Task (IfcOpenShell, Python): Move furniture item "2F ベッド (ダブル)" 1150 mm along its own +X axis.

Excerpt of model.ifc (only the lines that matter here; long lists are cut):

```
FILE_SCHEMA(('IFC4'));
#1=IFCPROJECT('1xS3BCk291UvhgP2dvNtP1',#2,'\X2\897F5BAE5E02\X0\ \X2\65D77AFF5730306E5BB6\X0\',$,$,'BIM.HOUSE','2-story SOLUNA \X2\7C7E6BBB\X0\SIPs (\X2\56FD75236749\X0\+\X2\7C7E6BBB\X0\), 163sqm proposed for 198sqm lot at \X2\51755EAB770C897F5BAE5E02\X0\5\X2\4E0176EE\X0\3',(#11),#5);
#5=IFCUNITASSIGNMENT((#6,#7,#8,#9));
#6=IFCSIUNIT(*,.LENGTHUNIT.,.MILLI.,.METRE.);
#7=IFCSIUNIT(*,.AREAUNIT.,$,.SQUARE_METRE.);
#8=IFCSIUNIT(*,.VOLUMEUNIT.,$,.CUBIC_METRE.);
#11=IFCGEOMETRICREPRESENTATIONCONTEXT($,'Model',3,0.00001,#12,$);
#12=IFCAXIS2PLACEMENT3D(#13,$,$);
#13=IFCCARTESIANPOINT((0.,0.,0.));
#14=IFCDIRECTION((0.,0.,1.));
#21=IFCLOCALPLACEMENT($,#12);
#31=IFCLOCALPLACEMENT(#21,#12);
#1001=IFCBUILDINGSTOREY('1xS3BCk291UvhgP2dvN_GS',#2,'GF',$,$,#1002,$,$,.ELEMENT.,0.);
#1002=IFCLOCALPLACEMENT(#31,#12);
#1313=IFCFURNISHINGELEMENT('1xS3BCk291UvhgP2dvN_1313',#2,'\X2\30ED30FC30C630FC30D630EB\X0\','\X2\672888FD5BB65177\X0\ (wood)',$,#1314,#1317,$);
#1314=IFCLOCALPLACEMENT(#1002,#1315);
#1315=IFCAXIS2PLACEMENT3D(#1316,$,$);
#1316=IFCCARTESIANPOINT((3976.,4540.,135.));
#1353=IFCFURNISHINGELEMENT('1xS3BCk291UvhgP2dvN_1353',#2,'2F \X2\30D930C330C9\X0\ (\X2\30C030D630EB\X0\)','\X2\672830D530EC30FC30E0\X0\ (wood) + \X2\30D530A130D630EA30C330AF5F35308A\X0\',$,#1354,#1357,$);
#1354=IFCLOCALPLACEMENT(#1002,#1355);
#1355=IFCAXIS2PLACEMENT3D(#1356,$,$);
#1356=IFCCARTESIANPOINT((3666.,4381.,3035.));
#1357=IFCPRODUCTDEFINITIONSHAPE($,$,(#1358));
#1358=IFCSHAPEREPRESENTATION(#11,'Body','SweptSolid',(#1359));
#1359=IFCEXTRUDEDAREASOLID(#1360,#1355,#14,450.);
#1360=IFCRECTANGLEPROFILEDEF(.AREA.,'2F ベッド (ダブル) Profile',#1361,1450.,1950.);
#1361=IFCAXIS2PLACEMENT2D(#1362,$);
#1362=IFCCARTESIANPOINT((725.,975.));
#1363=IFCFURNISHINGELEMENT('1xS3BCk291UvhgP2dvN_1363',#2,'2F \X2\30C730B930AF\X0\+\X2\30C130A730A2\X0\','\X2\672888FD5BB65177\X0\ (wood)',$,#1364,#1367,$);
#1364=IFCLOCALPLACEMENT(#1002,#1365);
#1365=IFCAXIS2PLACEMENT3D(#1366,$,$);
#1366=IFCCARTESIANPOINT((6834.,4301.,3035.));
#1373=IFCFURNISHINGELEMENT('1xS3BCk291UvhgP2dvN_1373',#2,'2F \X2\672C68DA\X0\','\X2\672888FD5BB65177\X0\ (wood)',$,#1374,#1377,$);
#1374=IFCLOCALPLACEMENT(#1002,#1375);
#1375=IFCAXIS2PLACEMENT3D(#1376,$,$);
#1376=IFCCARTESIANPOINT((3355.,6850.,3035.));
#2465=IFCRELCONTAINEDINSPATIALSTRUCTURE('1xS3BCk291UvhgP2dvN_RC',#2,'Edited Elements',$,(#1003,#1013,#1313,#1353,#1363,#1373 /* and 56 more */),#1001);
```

```python
import ifcopenshell
import ifcopenshell.api.geometry
import ifcopenshell.util.placement
import ifcopenshell.util.unit

model = ifcopenshell.open("model.ifc")
unit_scale = ifcopenshell.util.unit.calculate_unit_scale(model)

item = model.by_guid("1xS3BCk291UvhgP2dvN_1353")
matrix = ifcopenshell.util.placement.get_local_placement(item.ObjectPlacement)
matrix[:3, 3] += matrix[:3, 0] * 1.15 / unit_scale
ifcopenshell.api.geometry.edit_object_placement(model, product=item, matrix=matrix, is_si=False)

print(ifcopenshell.util.placement.get_local_placement(item.ObjectPlacement).round(3) + 0.0)

model.write("model_v2.ifc")
```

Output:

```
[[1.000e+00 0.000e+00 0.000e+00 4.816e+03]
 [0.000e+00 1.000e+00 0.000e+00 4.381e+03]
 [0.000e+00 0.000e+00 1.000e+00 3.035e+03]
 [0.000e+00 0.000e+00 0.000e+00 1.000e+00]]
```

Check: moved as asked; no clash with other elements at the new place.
